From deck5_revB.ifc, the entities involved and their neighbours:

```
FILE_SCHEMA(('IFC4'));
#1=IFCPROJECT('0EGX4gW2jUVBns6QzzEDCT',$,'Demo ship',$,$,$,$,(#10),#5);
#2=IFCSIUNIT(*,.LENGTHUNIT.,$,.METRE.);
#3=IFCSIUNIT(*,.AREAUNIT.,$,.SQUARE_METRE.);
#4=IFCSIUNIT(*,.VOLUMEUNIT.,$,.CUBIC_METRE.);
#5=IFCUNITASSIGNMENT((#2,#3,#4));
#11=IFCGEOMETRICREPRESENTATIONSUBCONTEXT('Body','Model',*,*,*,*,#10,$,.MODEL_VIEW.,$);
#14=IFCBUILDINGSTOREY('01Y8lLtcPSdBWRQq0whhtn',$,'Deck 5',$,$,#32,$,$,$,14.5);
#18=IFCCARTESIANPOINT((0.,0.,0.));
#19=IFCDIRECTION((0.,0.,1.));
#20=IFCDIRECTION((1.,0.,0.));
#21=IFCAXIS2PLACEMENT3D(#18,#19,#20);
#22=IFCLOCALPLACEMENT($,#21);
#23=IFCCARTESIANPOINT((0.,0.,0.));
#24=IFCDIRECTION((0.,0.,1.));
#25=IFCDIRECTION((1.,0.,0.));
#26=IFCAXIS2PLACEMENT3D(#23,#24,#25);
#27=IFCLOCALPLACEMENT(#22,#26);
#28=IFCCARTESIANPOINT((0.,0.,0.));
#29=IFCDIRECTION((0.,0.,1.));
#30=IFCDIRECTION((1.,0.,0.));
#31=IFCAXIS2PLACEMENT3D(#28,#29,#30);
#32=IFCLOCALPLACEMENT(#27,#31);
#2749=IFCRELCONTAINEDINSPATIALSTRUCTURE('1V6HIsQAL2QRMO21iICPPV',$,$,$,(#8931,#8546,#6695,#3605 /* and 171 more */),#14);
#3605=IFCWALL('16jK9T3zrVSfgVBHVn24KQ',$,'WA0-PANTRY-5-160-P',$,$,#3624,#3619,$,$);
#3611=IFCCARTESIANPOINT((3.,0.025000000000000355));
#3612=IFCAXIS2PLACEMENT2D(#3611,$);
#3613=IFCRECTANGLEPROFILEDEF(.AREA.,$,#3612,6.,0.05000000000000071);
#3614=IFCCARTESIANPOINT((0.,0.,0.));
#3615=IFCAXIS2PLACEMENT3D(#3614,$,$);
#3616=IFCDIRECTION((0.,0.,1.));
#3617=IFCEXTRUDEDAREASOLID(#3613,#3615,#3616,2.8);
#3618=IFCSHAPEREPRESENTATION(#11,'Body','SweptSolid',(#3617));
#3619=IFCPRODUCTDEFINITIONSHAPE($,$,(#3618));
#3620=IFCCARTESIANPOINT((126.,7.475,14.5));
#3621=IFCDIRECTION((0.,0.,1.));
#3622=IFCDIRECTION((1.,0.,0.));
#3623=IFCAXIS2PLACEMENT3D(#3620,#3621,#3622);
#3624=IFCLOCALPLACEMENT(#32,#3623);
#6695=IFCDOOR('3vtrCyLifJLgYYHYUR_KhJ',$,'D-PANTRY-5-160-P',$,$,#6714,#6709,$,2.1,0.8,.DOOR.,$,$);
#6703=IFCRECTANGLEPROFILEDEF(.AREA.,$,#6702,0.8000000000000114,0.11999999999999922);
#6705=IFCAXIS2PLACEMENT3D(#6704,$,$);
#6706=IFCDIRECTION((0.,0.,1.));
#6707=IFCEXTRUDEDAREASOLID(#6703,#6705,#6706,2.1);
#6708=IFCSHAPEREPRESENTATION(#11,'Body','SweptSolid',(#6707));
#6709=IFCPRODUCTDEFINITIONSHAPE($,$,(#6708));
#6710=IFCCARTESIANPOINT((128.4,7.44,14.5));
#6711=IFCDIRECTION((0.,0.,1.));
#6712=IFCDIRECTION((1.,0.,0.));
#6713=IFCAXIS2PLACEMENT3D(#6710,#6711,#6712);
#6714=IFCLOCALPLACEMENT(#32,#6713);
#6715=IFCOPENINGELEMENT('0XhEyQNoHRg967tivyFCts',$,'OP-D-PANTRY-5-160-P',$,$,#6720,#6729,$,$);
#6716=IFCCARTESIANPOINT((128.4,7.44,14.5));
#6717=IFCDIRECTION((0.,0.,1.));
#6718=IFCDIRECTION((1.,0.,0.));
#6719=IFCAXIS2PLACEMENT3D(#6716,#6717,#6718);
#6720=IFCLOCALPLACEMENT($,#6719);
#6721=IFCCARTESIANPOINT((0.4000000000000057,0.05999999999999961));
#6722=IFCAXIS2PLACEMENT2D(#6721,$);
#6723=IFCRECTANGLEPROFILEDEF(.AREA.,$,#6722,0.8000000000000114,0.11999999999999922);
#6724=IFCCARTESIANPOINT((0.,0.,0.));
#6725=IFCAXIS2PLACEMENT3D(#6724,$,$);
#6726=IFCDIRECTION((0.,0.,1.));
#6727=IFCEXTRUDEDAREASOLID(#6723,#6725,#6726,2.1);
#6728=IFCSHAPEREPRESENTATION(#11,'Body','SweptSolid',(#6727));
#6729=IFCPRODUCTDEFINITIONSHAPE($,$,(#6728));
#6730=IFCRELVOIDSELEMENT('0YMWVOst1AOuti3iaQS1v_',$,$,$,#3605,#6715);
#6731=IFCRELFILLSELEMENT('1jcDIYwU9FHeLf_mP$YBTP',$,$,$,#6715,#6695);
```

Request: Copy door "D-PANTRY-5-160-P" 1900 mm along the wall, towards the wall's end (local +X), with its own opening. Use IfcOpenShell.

```python
import ifcopenshell
import ifcopenshell.api.feature
import ifcopenshell.api.geometry
import ifcopenshell.api.root
import ifcopenshell.geom
import ifcopenshell.util.element
import ifcopenshell.util.placement
import ifcopenshell.util.shape
import ifcopenshell.util.unit

model = ifcopenshell.open("deck5_revB.ifc")
unit_scale = ifcopenshell.util.unit.calculate_unit_scale(model)
settings = ifcopenshell.geom.settings()


def volume(element):
    """Net volume in cubic metres, openings subtracted."""
    shape = ifcopenshell.geom.create_shape(settings, element)
    return ifcopenshell.util.shape.get_volume(shape.geometry)


door = model.by_id(6695)
opening = door.FillsVoids[0].RelatingOpeningElement
wall = opening.VoidsElements[0].RelatingBuildingElement
before = volume(wall)
shift = ifcopenshell.util.placement.get_local_placement(wall.ObjectPlacement)[:3, 0] * 1.9 / unit_scale

# copy_class copies the void relationship, type, container and properties, but no geometry.
new_opening = ifcopenshell.api.root.copy_class(model, product=opening)
new_opening.Representation = ifcopenshell.util.element.copy_deep(
    model, opening.Representation, exclude=["IfcGeometricRepresentationContext", "IfcRepresentationMap"]
)
new_door = ifcopenshell.api.root.copy_class(model, product=door)
new_door.Representation = ifcopenshell.util.element.copy_deep(
    model, door.Representation, exclude=["IfcGeometricRepresentationContext", "IfcRepresentationMap"]
)
ifcopenshell.api.feature.add_filling(model, opening=new_opening, element=new_door)

for old, new in ((opening, new_opening), (door, new_door)):
    matrix = ifcopenshell.util.placement.get_local_placement(old.ObjectPlacement)
    matrix[:3, 3] += shift
    ifcopenshell.api.geometry.edit_object_placement(model, product=new, matrix=matrix, is_si=False)

after = volume(wall)

print(f"wall volume {before:.3f} -> {after:.3f} m3")

model.write("deck5_revB-out.ifc")
```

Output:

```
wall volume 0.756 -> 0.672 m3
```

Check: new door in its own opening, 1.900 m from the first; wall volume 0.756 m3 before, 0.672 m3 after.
